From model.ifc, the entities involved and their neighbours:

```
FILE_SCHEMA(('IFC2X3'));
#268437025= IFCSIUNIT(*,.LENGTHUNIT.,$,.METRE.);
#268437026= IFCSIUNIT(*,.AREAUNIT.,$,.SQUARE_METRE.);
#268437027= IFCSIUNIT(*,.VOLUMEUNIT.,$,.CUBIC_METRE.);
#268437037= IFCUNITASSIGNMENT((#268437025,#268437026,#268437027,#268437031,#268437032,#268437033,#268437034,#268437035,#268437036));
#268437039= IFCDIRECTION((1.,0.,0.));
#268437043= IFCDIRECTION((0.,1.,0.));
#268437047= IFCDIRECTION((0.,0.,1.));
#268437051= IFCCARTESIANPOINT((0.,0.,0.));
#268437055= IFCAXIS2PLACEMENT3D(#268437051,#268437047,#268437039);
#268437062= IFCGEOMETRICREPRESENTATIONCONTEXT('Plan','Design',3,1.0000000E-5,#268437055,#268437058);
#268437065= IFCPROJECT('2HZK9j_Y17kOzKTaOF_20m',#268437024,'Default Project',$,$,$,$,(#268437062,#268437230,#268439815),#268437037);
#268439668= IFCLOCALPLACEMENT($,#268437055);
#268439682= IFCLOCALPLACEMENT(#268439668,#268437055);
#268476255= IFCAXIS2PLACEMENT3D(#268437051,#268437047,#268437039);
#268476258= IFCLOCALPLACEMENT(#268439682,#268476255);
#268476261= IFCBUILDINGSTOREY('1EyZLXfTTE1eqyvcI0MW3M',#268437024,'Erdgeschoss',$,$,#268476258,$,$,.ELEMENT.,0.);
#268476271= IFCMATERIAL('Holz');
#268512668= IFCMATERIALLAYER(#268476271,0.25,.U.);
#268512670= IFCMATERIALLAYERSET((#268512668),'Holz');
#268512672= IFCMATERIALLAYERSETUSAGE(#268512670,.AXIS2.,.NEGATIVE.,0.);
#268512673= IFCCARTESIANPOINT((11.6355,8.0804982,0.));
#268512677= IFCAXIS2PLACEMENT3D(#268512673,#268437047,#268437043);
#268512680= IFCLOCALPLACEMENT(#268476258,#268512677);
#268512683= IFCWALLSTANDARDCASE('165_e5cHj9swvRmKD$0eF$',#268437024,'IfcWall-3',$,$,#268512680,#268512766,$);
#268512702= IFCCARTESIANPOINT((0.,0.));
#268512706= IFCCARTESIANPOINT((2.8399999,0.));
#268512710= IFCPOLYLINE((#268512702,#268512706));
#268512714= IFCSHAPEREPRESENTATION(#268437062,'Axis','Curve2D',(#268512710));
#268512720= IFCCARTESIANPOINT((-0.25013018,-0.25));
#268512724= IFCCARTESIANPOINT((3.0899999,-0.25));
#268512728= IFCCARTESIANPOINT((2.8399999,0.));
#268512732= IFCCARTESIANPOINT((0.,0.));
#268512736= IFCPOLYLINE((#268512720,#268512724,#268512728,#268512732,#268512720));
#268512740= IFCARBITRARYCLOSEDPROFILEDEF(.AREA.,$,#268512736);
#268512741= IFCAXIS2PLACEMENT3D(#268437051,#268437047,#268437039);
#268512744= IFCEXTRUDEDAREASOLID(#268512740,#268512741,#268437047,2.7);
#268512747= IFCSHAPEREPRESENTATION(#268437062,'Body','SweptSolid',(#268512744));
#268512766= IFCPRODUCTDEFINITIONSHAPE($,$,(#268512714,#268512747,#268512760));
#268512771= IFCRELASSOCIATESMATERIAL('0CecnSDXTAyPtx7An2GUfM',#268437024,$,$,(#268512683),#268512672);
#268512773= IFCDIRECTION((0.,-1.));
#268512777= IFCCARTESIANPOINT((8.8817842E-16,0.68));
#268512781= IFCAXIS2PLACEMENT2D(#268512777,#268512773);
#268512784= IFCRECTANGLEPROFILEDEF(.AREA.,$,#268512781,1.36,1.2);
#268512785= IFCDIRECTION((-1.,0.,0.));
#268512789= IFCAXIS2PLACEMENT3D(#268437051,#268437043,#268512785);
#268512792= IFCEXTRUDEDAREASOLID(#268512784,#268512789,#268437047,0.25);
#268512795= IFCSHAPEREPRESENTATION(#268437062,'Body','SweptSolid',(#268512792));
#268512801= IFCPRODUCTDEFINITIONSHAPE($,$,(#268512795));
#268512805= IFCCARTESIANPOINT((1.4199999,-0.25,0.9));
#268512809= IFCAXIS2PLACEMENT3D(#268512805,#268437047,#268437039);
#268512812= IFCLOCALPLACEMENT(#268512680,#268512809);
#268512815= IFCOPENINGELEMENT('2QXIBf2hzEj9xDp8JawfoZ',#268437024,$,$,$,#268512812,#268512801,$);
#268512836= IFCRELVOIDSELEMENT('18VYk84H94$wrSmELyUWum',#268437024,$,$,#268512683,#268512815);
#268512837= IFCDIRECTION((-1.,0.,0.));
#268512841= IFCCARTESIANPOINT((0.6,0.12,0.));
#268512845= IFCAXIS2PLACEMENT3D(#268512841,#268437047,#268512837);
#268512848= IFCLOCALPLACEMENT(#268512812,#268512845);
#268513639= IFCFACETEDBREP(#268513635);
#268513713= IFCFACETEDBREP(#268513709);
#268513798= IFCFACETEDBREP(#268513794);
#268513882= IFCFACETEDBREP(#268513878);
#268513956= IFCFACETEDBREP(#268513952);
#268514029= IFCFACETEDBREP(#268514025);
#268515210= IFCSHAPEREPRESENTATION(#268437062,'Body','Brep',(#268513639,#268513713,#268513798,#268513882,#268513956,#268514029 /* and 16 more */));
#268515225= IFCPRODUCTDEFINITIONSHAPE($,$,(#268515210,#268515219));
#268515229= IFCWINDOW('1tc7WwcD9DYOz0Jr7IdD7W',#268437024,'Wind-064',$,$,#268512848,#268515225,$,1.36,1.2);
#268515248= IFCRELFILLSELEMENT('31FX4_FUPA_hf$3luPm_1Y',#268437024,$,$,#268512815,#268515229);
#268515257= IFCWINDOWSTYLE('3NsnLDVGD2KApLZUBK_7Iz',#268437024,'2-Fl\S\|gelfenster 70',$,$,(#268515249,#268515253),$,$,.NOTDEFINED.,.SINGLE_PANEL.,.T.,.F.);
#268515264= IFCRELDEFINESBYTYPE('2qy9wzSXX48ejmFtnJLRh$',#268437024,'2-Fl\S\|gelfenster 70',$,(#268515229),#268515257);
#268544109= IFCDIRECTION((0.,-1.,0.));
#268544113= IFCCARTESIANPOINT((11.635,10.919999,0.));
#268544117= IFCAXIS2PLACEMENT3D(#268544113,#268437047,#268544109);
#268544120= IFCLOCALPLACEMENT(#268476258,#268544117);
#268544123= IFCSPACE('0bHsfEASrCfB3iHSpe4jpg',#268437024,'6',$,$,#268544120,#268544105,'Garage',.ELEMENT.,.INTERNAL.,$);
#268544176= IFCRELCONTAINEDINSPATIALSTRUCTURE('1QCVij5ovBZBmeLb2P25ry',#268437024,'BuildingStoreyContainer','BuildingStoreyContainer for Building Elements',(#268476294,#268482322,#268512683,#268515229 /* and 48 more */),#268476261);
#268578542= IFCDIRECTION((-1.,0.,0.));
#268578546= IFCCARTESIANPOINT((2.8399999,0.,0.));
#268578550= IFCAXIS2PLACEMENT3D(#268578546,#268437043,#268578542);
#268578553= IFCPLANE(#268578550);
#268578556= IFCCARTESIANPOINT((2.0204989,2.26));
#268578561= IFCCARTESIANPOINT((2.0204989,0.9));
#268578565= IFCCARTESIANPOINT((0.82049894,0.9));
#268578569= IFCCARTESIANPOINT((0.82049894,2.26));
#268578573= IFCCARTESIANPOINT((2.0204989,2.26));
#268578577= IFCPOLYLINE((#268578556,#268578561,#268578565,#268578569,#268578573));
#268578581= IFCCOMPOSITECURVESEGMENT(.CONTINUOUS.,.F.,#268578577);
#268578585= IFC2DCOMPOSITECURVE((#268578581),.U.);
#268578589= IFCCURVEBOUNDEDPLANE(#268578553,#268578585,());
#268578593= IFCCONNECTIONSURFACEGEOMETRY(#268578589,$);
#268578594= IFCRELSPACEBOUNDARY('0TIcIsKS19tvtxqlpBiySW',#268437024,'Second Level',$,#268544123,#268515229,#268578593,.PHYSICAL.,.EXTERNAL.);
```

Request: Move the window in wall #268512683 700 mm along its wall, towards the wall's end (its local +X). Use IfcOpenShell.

```python
import numpy as np
import ifcopenshell
import ifcopenshell.api.geometry
import ifcopenshell.util.placement
import ifcopenshell.util.unit

model = ifcopenshell.open("model.ifc")
unit_scale = ifcopenshell.util.unit.calculate_unit_scale(model)

window = model.by_guid("1tc7WwcD9DYOz0Jr7IdD7W")
opening = window.FillsVoids[0].RelatingOpeningElement
wall = opening.VoidsElements[0].RelatingBuildingElement

wall_matrix = ifcopenshell.util.placement.get_local_placement(wall.ObjectPlacement)
shift = wall_matrix[:3, 0] * 0.7 / unit_scale
before = ifcopenshell.util.placement.get_local_placement(window.ObjectPlacement)[:3, 3].copy()

# The window is placed relative to its opening, so it follows when the opening moves.
matrix = ifcopenshell.util.placement.get_local_placement(opening.ObjectPlacement)
matrix[:3, 3] += shift
ifcopenshell.api.geometry.edit_object_placement(
    model, product=opening, matrix=matrix, is_si=False, should_transform_children=True
)

# Space boundary surfaces are stored in each space's coordinates; move them too.
for rel in window.ProvidesBoundaries:
    if not rel.ConnectionGeometry:
        continue
    surface = rel.ConnectionGeometry.SurfaceOnRelatingElement.BasisSurface
    space_matrix = ifcopenshell.util.placement.get_local_placement(rel.RelatingSpace.ObjectPlacement)
    point = np.array(surface.Position.Location.Coordinates) + space_matrix[:3, :3].T @ shift
    surface.Position = model.createIfcAxis2Placement3D(
        model.createIfcCartesianPoint(point.tolist()), surface.Position.Axis, surface.Position.RefDirection
    )

after = ifcopenshell.util.placement.get_local_placement(window.ObjectPlacement)[:3, 3]
print("window moved by", (after - before).round(3) + 0.0)

model.write("model_updated.ifc")
```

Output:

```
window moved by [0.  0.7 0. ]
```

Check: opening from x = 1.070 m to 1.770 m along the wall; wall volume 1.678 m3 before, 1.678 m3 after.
